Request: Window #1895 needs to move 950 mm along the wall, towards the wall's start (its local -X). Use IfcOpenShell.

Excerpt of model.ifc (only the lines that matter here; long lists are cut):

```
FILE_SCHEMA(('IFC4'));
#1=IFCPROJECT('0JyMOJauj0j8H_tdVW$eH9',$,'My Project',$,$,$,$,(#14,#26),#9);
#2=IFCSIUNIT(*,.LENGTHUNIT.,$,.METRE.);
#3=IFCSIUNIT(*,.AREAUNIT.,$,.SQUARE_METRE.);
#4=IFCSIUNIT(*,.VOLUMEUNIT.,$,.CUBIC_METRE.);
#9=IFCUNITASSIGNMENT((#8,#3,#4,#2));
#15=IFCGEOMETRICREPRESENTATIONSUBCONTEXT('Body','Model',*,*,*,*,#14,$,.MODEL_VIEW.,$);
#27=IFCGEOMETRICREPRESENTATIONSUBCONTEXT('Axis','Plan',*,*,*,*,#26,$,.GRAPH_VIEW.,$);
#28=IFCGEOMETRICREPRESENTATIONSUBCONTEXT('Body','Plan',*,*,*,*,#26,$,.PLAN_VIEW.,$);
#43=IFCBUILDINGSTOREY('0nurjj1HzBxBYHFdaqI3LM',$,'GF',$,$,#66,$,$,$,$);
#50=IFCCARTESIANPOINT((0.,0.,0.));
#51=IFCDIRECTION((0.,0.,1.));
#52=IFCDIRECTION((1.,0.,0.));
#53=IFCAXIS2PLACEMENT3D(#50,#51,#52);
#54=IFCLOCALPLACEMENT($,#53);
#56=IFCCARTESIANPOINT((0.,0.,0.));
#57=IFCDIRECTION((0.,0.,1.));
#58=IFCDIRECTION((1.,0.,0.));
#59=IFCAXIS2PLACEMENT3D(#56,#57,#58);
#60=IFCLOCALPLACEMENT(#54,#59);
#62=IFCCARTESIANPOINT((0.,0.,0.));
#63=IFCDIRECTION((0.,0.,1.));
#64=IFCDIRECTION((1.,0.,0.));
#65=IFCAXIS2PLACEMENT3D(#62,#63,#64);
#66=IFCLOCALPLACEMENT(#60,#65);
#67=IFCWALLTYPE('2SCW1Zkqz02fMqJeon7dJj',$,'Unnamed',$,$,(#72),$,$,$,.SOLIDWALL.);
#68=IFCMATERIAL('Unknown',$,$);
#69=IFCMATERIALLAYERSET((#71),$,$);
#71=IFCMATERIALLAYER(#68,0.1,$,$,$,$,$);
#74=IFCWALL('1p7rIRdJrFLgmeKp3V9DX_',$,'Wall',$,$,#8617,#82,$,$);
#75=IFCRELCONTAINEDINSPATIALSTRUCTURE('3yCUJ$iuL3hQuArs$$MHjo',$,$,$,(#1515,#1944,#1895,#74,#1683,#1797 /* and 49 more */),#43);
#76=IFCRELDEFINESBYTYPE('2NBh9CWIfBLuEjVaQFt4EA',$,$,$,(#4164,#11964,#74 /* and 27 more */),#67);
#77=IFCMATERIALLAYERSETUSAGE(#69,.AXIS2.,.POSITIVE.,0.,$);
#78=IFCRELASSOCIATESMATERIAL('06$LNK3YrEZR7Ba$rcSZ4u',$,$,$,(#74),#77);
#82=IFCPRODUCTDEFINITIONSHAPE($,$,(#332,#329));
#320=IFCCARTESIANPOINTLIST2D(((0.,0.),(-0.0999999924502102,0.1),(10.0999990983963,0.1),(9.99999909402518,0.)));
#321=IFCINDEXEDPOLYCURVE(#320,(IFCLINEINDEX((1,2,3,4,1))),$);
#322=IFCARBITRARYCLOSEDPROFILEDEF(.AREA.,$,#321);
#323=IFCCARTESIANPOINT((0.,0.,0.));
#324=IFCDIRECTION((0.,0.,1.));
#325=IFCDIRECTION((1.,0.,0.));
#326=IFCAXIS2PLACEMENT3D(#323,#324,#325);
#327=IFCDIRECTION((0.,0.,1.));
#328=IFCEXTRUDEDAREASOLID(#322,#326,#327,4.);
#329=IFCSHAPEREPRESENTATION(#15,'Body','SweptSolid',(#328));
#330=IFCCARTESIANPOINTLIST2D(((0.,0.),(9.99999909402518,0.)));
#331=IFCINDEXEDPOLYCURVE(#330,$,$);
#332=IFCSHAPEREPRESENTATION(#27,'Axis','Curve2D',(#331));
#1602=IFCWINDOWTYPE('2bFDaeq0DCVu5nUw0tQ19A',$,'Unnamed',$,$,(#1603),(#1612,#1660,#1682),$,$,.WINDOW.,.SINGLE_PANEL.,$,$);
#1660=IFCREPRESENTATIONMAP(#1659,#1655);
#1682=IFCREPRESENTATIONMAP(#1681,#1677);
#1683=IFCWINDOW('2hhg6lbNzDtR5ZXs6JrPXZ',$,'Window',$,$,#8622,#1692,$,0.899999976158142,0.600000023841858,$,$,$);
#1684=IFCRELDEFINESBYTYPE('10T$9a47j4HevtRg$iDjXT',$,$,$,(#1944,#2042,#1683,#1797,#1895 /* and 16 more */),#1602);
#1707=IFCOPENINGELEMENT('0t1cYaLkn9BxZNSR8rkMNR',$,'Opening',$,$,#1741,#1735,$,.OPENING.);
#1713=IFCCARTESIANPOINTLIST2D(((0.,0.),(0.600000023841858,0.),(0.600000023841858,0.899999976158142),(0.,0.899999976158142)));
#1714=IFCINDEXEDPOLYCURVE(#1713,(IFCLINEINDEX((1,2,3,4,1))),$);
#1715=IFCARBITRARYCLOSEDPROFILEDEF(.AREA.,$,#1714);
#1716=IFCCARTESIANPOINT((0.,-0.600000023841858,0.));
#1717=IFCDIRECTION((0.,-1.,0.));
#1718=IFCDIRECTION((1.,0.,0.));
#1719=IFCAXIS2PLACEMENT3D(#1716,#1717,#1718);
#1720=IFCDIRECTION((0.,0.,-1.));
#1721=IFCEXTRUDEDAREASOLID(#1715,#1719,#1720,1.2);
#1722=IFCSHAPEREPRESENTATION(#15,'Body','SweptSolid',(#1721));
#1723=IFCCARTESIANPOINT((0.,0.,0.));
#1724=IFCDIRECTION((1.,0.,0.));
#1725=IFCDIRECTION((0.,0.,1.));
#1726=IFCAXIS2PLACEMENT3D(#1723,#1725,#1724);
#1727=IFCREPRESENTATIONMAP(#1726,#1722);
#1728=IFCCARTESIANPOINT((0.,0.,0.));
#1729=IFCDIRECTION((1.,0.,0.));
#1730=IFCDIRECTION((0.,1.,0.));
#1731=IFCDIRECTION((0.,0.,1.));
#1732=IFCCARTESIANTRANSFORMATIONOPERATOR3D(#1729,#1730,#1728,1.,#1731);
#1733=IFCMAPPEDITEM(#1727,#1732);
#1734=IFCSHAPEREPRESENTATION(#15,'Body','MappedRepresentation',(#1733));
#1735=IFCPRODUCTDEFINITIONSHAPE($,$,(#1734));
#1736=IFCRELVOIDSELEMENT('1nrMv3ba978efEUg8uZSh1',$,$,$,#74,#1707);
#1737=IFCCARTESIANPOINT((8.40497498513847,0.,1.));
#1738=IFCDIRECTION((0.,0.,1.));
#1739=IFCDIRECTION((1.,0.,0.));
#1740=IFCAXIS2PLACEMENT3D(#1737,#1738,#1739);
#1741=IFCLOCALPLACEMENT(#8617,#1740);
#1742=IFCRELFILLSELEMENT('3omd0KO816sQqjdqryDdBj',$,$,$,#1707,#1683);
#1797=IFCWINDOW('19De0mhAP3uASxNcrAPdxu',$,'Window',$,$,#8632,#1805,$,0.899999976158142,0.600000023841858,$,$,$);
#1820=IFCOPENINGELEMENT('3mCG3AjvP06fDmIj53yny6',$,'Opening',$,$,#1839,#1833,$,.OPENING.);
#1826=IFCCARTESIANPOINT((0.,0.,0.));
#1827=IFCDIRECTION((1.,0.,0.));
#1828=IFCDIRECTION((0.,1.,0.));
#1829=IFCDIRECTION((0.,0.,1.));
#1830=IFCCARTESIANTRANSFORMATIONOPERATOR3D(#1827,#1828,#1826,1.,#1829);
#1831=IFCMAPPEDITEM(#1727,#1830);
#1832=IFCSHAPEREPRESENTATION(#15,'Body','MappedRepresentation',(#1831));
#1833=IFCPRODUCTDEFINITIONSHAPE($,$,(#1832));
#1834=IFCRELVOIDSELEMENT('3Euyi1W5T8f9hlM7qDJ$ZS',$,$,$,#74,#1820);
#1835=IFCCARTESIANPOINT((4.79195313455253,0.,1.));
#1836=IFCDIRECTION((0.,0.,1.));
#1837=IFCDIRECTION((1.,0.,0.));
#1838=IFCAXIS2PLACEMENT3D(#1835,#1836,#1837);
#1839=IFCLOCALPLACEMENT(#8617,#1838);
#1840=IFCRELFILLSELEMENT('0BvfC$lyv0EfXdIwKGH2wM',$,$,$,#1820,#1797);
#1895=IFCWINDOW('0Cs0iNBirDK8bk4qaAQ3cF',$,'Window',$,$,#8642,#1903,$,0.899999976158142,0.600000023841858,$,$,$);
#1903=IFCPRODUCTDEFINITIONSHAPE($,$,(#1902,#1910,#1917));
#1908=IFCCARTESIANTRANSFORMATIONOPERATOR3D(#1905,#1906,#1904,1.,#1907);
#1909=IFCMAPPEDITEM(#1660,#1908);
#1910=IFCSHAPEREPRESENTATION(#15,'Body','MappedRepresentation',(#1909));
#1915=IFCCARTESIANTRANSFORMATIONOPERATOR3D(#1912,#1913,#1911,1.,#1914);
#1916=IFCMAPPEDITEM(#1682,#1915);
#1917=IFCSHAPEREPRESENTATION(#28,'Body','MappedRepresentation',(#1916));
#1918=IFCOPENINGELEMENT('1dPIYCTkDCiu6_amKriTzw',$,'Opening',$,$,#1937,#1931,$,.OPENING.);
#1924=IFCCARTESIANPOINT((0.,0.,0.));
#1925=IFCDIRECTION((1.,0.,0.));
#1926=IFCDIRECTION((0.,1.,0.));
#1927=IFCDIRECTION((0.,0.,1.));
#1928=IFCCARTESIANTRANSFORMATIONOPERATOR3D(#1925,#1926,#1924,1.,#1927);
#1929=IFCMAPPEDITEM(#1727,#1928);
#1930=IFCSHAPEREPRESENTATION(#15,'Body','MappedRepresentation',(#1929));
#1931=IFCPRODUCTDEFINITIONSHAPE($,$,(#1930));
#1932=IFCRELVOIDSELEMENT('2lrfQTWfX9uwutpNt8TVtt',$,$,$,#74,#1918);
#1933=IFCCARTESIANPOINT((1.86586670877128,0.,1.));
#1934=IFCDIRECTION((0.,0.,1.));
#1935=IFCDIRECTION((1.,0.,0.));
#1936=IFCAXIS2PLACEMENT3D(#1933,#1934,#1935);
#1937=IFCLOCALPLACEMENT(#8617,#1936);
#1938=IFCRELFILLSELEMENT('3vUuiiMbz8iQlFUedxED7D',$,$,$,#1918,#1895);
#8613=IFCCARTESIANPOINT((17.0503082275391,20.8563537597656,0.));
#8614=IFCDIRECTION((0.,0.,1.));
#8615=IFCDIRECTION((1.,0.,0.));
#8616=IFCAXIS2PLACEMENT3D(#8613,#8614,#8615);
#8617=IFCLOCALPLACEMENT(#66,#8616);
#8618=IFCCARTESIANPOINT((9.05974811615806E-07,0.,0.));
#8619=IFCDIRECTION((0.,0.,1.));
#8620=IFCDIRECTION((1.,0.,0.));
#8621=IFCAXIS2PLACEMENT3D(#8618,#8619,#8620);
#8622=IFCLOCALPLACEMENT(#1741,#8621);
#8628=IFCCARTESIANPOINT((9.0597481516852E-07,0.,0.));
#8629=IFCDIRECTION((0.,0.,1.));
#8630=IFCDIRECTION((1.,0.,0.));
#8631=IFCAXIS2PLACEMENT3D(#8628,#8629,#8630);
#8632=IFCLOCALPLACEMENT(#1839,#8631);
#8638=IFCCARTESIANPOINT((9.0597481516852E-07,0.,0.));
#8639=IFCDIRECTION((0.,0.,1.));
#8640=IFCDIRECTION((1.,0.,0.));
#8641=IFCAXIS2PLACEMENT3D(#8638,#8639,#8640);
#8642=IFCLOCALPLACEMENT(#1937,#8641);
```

```python
import ifcopenshell
import ifcopenshell.api.geometry
import ifcopenshell.util.placement
import ifcopenshell.util.unit

model = ifcopenshell.open("model.ifc")
unit_scale = ifcopenshell.util.unit.calculate_unit_scale(model)

window = model.by_guid("0Cs0iNBirDK8bk4qaAQ3cF")
opening = window.FillsVoids[0].RelatingOpeningElement
wall = opening.VoidsElements[0].RelatingBuildingElement

wall_matrix = ifcopenshell.util.placement.get_local_placement(wall.ObjectPlacement)
shift = wall_matrix[:3, 0] * -0.95 / unit_scale
before = ifcopenshell.util.placement.get_local_placement(window.ObjectPlacement)[:3, 3].copy()

# The window is placed relative to its opening, so it follows when the opening moves.
matrix = ifcopenshell.util.placement.get_local_placement(opening.ObjectPlacement)
matrix[:3, 3] += shift
ifcopenshell.api.geometry.edit_object_placement(
    model, product=opening, matrix=matrix, is_si=False, should_transform_children=True
)

after = ifcopenshell.util.placement.get_local_placement(window.ObjectPlacement)[:3, 3]
print("window moved by", (after - before).round(3) + 0.0)

model.write("model_v2.ifc")
```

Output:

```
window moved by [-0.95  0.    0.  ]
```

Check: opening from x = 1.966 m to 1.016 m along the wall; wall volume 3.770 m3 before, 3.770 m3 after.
